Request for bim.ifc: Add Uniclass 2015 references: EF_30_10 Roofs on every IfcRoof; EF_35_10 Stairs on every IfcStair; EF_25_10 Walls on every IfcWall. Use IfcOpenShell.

First a look at what the model holds.

```python
import ifcopenshell

model = ifcopenshell.open("bim.ifc")
print(model.schema)
print("classifications:", [c.Name for c in model.by_type("IfcClassification")])
for ifc_class in ("IfcDoor", "IfcRoof", "IfcStair", "IfcWall", "IfcWindow"):
    print(ifc_class, len(model.by_type(ifc_class)))
```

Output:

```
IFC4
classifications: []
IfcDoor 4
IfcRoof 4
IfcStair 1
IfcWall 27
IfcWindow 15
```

```python
import ifcopenshell
import ifcopenshell.api.classification

model = ifcopenshell.open("bim.ifc")

system = ifcopenshell.api.classification.add_classification(model, classification="Uniclass 2015")

codes = {
    "IfcRoof": ("EF_30_10", "Roofs"),
    "IfcStair": ("EF_35_10", "Stairs"),
    "IfcWall": ("EF_25_10", "Walls"),
}
for ifc_class, (code, name) in codes.items():
    products = model.by_type(ifc_class)
    ifcopenshell.api.classification.add_reference(
        model, products=products, classification=system, identification=code, name=name
    )
    print(code, len(products))

model.write("bim-out.ifc")
```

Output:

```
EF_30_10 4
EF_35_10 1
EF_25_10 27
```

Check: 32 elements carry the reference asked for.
